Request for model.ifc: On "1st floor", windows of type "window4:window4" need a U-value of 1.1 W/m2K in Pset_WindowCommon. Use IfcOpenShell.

First a look at what the model holds.

```python
import ifcopenshell
import ifcopenshell.util.element

model = ifcopenshell.open("model.ifc")
print(model.schema)
storey = next(s for s in model.by_type("IfcBuildingStorey") if s.Name == "1st floor")
windows = [e for e in ifcopenshell.util.element.get_decomposition(storey) if e.is_a("IfcWindow")]
seen = {}
for e in windows:
    element_type = ifcopenshell.util.element.get_type(e)
    key = (element_type.Name if element_type != e and element_type else None, ifcopenshell.util.element.get_pset(e, "Pset_WindowCommon", "ThermalTransmittance"))
    seen[key] = seen.get(key, 0) + 1
for (name, value), count in sorted(seen.items(), key=str):
    print(count, "x", name, "|", value)
```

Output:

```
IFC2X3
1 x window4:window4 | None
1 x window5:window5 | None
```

```python
import ifcopenshell
import ifcopenshell.api.pset
import ifcopenshell.util.element

model = ifcopenshell.open("model.ifc")

storey = next(s for s in model.by_type("IfcBuildingStorey") if s.Name == "1st floor")
windows = [e for e in ifcopenshell.util.element.get_decomposition(storey) if e.is_a("IfcWindow")]

count = 0
for e in windows:
    element_type = ifcopenshell.util.element.get_type(e)
    if element_type in (None, e) or element_type.Name != "window4:window4":
        continue
    # add_pset returns the element's existing set when there is one.
    pset = ifcopenshell.api.pset.add_pset(model, product=e, name="Pset_WindowCommon")
    ifcopenshell.api.pset.edit_pset(model, pset=pset, properties={"ThermalTransmittance": 1.1})
    count += 1

print(count, "windows updated")

model.write("model_rev.ifc")
```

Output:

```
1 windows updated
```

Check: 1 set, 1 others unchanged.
